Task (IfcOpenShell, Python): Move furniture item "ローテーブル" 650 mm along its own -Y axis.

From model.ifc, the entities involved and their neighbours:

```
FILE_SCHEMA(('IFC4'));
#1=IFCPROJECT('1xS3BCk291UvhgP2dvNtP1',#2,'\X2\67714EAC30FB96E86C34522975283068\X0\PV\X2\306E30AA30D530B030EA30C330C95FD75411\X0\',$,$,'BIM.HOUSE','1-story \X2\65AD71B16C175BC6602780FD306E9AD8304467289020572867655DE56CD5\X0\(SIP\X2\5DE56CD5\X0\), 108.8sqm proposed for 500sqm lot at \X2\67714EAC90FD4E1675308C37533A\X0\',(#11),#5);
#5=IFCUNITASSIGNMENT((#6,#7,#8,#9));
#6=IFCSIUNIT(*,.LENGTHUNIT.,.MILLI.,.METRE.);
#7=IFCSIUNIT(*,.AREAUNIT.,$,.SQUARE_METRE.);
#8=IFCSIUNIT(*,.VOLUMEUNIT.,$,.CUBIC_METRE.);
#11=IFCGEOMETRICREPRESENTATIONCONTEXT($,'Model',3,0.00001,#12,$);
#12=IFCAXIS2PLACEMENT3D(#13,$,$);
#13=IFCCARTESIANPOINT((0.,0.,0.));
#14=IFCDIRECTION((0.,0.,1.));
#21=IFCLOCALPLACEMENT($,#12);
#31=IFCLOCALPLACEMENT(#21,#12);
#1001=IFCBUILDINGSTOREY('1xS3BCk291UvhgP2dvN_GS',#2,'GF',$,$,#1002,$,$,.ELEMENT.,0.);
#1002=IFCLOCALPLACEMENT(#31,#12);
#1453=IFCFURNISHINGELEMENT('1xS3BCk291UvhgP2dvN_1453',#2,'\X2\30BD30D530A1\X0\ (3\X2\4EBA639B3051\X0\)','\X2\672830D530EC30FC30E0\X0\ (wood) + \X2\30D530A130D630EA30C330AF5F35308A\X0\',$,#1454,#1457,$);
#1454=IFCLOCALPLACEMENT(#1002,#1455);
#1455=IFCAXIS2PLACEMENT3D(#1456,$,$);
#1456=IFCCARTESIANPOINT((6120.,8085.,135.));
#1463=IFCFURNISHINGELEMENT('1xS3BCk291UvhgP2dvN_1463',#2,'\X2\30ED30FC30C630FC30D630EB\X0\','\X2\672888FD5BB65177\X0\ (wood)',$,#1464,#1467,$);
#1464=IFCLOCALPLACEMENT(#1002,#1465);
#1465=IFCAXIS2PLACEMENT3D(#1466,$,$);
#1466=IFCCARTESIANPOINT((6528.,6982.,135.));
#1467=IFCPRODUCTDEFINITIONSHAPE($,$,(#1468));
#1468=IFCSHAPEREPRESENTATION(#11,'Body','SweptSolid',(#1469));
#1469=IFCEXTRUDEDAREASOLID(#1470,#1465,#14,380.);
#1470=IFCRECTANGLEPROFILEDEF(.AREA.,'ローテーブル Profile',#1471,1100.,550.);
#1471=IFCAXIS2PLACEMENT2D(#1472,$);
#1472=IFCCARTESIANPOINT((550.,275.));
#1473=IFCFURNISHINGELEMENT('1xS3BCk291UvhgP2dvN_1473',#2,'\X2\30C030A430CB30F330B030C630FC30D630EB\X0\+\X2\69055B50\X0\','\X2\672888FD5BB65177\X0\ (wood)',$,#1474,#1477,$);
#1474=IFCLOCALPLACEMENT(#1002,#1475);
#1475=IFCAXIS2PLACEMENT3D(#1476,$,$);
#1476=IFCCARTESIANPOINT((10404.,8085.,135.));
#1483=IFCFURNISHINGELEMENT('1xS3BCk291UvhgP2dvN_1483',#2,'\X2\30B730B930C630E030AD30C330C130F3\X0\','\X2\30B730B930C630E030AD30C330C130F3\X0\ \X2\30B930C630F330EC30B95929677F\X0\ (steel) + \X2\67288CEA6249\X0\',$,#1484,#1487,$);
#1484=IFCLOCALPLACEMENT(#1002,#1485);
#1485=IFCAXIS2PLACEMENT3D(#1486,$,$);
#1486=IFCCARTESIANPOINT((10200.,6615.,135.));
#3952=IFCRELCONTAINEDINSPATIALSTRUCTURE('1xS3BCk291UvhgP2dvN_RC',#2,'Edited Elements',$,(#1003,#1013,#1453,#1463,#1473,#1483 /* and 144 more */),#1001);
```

```python
import ifcopenshell
import ifcopenshell.api.geometry
import ifcopenshell.util.placement
import ifcopenshell.util.unit

model = ifcopenshell.open("model.ifc")
unit_scale = ifcopenshell.util.unit.calculate_unit_scale(model)

item = model.by_guid("1xS3BCk291UvhgP2dvN_1463")
matrix = ifcopenshell.util.placement.get_local_placement(item.ObjectPlacement)
matrix[:3, 3] -= matrix[:3, 1] * 0.65 / unit_scale
ifcopenshell.api.geometry.edit_object_placement(model, product=item, matrix=matrix, is_si=False)

print(ifcopenshell.util.placement.get_local_placement(item.ObjectPlacement).round(3) + 0.0)

model.write("model_v2.ifc")
```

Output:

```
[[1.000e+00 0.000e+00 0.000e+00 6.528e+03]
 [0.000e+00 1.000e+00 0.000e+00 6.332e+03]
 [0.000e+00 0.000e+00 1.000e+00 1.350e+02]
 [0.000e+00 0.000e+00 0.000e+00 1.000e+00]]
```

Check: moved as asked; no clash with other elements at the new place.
